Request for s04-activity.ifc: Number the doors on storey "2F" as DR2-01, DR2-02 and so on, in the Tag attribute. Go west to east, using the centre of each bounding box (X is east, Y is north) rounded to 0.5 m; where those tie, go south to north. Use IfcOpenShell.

First a look at what the model holds.

```python
import ifcopenshell
import ifcopenshell.util.element
import ifcopenshell.util.placement

model = ifcopenshell.open("s04-activity.ifc")
print(model.schema)
storey = next(s for s in model.by_type("IfcBuildingStorey") if s.Name == "2F")
doors = [e for e in ifcopenshell.util.element.get_decomposition(storey) if e.is_a("IfcDoor")]
for e in sorted(doors, key=lambda e: e.id()):
    origin = ifcopenshell.util.placement.get_local_placement(e.ObjectPlacement)[:3, 3]
    print(e.id(), e.Tag, e.Name, origin.round(2) + 0.0, sep=" | ")
```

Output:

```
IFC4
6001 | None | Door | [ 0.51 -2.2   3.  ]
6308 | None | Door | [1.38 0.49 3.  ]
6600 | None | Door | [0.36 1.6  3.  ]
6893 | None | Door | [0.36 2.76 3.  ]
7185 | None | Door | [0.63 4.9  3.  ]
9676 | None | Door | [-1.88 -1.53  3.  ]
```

```python
import ifcopenshell
import ifcopenshell.geom
import ifcopenshell.util.element
import ifcopenshell.util.shape

model = ifcopenshell.open("s04-activity.ifc")
settings = ifcopenshell.geom.settings()
settings.set("use-world-coords", True)


def centre(element):
    shape = ifcopenshell.geom.create_shape(settings, element)
    return ifcopenshell.util.shape.get_bbox_centroid(shape.geometry)


storey = next(s for s in model.by_type("IfcBuildingStorey") if s.Name == "2F")
doors = [e for e in ifcopenshell.util.element.get_decomposition(storey) if e.is_a("IfcDoor")]

# Insertion points can sit at a corner or the storey origin, so sort by the geometry (in metres).
centres = {e: centre(e) for e in doors}
doors.sort(key=lambda e: (round(centres[e][0] / 0.5), centres[e][1]))

for i, e in enumerate(doors, start=1):
    number = f"DR2-{i:02d}"
    e.Tag = number
    print(e.id(), number)

model.write("s04-activity_edited.ifc")
```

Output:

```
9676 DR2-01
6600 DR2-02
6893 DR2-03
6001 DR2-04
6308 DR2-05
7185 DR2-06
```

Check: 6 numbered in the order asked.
